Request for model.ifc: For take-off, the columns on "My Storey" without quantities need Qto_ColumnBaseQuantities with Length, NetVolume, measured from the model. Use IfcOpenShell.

First a look at what the model holds.

```python
import ifcopenshell
import ifcopenshell.util.element
import ifcopenshell.util.unit

model = ifcopenshell.open("model.ifc")
print(model.schema)
for unit_type in ("LENGTHUNIT", "AREAUNIT", "VOLUMEUNIT"):
    print(unit_type, ifcopenshell.util.unit.calculate_unit_scale(model, unit_type))
storey = next(s for s in model.by_type("IfcBuildingStorey") if s.Name == "My Storey")
columns = [e for e in ifcopenshell.util.element.get_decomposition(storey) if e.is_a("IfcColumn")]
for e in sorted(columns, key=lambda e: e.id()):
    print(e.id(), e.is_a(), e.Name, list(ifcopenshell.util.element.get_psets(e, qtos_only=True)), sep=" | ")
```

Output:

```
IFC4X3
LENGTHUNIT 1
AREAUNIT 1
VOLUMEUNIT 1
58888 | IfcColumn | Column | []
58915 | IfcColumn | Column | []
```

```python
import ifcopenshell
import ifcopenshell.api.pset
import ifcopenshell.geom
import ifcopenshell.util.element
import ifcopenshell.util.shape
import ifcopenshell.util.unit

model = ifcopenshell.open("model.ifc")
unit_scale = ifcopenshell.util.unit.calculate_unit_scale(model)
volume_scale = ifcopenshell.util.unit.calculate_unit_scale(model, "VOLUMEUNIT")
settings = ifcopenshell.geom.settings()

storey = next(s for s in model.by_type("IfcBuildingStorey") if s.Name == "My Storey")
columns = [e for e in ifcopenshell.util.element.get_decomposition(storey) if e.is_a("IfcColumn")]

for e in sorted(columns, key=lambda e: e.id()):
    if ifcopenshell.util.element.get_psets(e, qtos_only=True, should_inherit=False):
        continue
    # Geometry comes back in metres, in the element's own axes.
    shape = ifcopenshell.geom.create_shape(settings, e)
    values = {
        "Length": ifcopenshell.util.shape.get_z(shape.geometry) / unit_scale,
        "NetVolume": ifcopenshell.util.shape.get_volume(shape.geometry) / volume_scale,
    }
    qto = ifcopenshell.api.pset.add_qto(model, product=e, name="Qto_ColumnBaseQuantities")
    ifcopenshell.api.pset.edit_qto(model, qto=qto, properties=values)
    print(e.id(), {k: round(v, 3) for k, v in values.items()})

model.write("model-out.ifc")
```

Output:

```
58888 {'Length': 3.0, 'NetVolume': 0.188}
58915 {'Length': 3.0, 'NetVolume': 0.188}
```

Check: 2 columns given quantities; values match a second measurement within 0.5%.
